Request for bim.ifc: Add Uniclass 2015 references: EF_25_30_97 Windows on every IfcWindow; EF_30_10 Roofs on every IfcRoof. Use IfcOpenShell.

First a look at what the model holds.

```python
import ifcopenshell

model = ifcopenshell.open("bim.ifc")
print(model.schema)
print("classifications:", [c.Name for c in model.by_type("IfcClassification")])
for ifc_class in ("IfcDoor", "IfcRoof", "IfcStair", "IfcWall", "IfcWindow"):
    print(ifc_class, len(model.by_type(ifc_class)))
```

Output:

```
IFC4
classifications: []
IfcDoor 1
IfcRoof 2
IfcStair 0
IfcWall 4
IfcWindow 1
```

```python
import ifcopenshell
import ifcopenshell.api.classification

model = ifcopenshell.open("bim.ifc")

system = ifcopenshell.api.classification.add_classification(model, classification="Uniclass 2015")

codes = {
    "IfcWindow": ("EF_25_30_97", "Windows"),
    "IfcRoof": ("EF_30_10", "Roofs"),
}
for ifc_class, (code, name) in codes.items():
    products = model.by_type(ifc_class)
    ifcopenshell.api.classification.add_reference(
        model, products=products, classification=system, identification=code, name=name
    )
    print(code, len(products))

model.write("bim_edited.ifc")
```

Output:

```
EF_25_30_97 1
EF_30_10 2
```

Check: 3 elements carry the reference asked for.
